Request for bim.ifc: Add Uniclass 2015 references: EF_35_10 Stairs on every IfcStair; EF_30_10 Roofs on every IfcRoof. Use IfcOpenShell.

First a look at what the model holds.

```python
import ifcopenshell

model = ifcopenshell.open("bim.ifc")
print(model.schema)
print("classifications:", [c.Name for c in model.by_type("IfcClassification")])
for ifc_class in ("IfcDoor", "IfcRoof", "IfcStair", "IfcWall", "IfcWindow"):
    print(ifc_class, len(model.by_type(ifc_class)))
```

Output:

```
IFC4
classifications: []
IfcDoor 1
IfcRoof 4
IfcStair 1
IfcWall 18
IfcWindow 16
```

```python
import ifcopenshell
import ifcopenshell.api.classification

model = ifcopenshell.open("bim.ifc")

system = ifcopenshell.api.classification.add_classification(model, classification="Uniclass 2015")

codes = {
    "IfcStair": ("EF_35_10", "Stairs"),
    "IfcRoof": ("EF_30_10", "Roofs"),
}
for ifc_class, (code, name) in codes.items():
    products = model.by_type(ifc_class)
    ifcopenshell.api.classification.add_reference(
        model, products=products, classification=system, identification=code, name=name
    )
    print(code, len(products))

model.write("bim_edited.ifc")
```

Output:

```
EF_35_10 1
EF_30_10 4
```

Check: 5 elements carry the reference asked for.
